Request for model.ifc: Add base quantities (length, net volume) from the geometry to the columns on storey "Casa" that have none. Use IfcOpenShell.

First a look at what the model holds.

```python
import ifcopenshell
import ifcopenshell.util.element
import ifcopenshell.util.unit

model = ifcopenshell.open("model.ifc")
print(model.schema)
for unit_type in ("LENGTHUNIT", "AREAUNIT", "VOLUMEUNIT"):
    print(unit_type, ifcopenshell.util.unit.calculate_unit_scale(model, unit_type))
storey = next(s for s in model.by_type("IfcBuildingStorey") if s.Name == "Casa")
columns = [e for e in ifcopenshell.util.element.get_decomposition(storey) if e.is_a("IfcColumn")]
for e in sorted(columns, key=lambda e: e.id()):
    print(e.id(), e.is_a(), e.Name, list(ifcopenshell.util.element.get_psets(e, qtos_only=True)), sep=" | ")
```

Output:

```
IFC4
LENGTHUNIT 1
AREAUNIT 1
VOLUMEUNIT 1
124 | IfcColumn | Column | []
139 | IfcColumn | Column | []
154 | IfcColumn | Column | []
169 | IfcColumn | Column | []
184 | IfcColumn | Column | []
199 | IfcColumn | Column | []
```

```python
import ifcopenshell
import ifcopenshell.api.pset
import ifcopenshell.geom
import ifcopenshell.util.element
import ifcopenshell.util.shape
import ifcopenshell.util.unit

model = ifcopenshell.open("model.ifc")
unit_scale = ifcopenshell.util.unit.calculate_unit_scale(model)
volume_scale = ifcopenshell.util.unit.calculate_unit_scale(model, "VOLUMEUNIT")
settings = ifcopenshell.geom.settings()

storey = next(s for s in model.by_type("IfcBuildingStorey") if s.Name == "Casa")
columns = [e for e in ifcopenshell.util.element.get_decomposition(storey) if e.is_a("IfcColumn")]

for e in sorted(columns, key=lambda e: e.id()):
    if ifcopenshell.util.element.get_psets(e, qtos_only=True, should_inherit=False):
        continue
    # Geometry comes back in metres, in the element's own axes.
    shape = ifcopenshell.geom.create_shape(settings, e)
    values = {
        "Length": ifcopenshell.util.shape.get_z(shape.geometry) / unit_scale,
        "NetVolume": ifcopenshell.util.shape.get_volume(shape.geometry) / volume_scale,
    }
    qto = ifcopenshell.api.pset.add_qto(model, product=e, name="Qto_ColumnBaseQuantities")
    ifcopenshell.api.pset.edit_qto(model, qto=qto, properties=values)
    print(e.id(), {k: round(v, 3) for k, v in values.items()})

model.write("model_v2.ifc")
```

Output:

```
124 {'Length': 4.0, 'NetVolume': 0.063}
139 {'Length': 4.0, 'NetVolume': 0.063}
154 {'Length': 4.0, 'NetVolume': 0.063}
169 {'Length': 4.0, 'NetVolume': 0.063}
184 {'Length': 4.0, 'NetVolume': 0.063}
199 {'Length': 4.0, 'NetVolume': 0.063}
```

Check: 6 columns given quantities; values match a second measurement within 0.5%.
